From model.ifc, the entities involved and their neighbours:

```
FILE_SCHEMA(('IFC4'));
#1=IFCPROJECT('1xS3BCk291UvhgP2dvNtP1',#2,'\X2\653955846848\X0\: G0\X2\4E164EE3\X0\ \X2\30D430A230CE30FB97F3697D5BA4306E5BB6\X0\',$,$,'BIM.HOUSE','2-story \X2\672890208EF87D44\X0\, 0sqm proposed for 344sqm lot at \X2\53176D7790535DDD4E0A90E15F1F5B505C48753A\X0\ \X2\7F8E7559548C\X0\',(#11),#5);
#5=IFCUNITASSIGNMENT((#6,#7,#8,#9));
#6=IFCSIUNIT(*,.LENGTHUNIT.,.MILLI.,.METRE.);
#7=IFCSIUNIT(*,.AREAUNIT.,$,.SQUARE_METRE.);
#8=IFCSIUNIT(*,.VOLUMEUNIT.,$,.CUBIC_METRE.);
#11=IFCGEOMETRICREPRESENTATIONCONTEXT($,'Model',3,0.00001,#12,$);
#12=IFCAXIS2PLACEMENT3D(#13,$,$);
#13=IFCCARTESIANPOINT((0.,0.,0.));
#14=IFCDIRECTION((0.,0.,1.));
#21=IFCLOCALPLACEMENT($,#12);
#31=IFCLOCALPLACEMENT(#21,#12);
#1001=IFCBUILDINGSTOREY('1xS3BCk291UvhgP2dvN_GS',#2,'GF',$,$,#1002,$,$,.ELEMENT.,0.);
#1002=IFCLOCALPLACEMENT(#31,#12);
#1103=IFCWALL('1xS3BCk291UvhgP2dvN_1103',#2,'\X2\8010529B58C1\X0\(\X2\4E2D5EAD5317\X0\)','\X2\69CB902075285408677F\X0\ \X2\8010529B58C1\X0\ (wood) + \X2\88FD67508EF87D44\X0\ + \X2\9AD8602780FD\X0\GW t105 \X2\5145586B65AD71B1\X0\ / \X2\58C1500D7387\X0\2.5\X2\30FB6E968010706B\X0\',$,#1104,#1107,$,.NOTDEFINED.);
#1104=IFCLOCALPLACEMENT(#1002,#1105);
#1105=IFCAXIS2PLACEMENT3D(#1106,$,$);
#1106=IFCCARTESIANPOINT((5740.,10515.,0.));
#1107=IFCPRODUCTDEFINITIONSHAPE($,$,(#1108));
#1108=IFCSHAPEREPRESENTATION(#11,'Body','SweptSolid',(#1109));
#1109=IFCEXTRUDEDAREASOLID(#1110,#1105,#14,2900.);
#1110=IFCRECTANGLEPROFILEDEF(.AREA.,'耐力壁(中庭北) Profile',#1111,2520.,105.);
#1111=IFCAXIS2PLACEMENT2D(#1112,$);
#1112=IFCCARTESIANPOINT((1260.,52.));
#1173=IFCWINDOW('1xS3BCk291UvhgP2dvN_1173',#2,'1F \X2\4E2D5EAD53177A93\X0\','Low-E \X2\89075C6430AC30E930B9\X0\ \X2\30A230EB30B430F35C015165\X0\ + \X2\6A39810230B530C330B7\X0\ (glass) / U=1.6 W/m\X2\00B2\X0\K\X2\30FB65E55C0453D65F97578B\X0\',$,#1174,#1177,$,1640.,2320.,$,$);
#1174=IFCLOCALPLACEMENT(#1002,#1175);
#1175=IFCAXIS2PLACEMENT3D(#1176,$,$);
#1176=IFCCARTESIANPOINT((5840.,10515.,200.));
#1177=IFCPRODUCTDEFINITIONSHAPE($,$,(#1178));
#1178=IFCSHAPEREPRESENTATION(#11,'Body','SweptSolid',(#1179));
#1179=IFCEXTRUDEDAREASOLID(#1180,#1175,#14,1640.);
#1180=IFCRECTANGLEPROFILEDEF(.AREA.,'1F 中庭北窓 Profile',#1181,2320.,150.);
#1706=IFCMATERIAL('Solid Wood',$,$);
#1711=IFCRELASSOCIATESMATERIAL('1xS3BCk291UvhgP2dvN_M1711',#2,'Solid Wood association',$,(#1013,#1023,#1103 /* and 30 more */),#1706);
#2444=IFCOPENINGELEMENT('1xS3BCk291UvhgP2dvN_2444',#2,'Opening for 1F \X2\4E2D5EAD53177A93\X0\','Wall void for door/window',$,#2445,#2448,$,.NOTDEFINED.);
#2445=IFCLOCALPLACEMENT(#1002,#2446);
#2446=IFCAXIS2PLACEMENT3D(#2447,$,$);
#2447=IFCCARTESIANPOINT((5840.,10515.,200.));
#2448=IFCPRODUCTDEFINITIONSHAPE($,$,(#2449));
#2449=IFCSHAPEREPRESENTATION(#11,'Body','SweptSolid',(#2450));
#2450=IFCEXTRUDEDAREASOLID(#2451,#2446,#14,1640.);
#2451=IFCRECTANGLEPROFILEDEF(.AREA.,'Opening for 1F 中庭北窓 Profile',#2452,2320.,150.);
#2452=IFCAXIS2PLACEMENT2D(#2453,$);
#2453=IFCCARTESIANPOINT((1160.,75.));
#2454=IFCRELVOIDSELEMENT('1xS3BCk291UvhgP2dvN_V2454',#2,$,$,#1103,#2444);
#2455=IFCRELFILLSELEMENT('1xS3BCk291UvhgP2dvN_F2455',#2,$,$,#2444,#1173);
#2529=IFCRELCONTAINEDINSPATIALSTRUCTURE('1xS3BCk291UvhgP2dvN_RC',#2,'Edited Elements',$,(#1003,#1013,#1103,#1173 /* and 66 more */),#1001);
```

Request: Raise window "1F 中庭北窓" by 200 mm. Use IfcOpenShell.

```python
import numpy as np
import ifcopenshell
import ifcopenshell.api.geometry
import ifcopenshell.util.placement
import ifcopenshell.util.unit

model = ifcopenshell.open("model.ifc")
unit_scale = ifcopenshell.util.unit.calculate_unit_scale(model)

window = model.by_guid("1xS3BCk291UvhgP2dvN_1173")
opening = window.FillsVoids[0].RelatingOpeningElement
dz = 0.2 / unit_scale

shift = np.array([0.0, 0.0, dz])
# The window is not placed relative to its opening, so move both.
for product in (opening, window):
    matrix = ifcopenshell.util.placement.get_local_placement(product.ObjectPlacement)
    matrix[:3, 3] += shift
    ifcopenshell.api.geometry.edit_object_placement(model, product=product, matrix=matrix, is_si=False)

print(f"moved by {dz * unit_scale:+.3f} m")

model.write("model_v2.ifc")
```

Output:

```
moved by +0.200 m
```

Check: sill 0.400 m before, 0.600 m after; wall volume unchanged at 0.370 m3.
